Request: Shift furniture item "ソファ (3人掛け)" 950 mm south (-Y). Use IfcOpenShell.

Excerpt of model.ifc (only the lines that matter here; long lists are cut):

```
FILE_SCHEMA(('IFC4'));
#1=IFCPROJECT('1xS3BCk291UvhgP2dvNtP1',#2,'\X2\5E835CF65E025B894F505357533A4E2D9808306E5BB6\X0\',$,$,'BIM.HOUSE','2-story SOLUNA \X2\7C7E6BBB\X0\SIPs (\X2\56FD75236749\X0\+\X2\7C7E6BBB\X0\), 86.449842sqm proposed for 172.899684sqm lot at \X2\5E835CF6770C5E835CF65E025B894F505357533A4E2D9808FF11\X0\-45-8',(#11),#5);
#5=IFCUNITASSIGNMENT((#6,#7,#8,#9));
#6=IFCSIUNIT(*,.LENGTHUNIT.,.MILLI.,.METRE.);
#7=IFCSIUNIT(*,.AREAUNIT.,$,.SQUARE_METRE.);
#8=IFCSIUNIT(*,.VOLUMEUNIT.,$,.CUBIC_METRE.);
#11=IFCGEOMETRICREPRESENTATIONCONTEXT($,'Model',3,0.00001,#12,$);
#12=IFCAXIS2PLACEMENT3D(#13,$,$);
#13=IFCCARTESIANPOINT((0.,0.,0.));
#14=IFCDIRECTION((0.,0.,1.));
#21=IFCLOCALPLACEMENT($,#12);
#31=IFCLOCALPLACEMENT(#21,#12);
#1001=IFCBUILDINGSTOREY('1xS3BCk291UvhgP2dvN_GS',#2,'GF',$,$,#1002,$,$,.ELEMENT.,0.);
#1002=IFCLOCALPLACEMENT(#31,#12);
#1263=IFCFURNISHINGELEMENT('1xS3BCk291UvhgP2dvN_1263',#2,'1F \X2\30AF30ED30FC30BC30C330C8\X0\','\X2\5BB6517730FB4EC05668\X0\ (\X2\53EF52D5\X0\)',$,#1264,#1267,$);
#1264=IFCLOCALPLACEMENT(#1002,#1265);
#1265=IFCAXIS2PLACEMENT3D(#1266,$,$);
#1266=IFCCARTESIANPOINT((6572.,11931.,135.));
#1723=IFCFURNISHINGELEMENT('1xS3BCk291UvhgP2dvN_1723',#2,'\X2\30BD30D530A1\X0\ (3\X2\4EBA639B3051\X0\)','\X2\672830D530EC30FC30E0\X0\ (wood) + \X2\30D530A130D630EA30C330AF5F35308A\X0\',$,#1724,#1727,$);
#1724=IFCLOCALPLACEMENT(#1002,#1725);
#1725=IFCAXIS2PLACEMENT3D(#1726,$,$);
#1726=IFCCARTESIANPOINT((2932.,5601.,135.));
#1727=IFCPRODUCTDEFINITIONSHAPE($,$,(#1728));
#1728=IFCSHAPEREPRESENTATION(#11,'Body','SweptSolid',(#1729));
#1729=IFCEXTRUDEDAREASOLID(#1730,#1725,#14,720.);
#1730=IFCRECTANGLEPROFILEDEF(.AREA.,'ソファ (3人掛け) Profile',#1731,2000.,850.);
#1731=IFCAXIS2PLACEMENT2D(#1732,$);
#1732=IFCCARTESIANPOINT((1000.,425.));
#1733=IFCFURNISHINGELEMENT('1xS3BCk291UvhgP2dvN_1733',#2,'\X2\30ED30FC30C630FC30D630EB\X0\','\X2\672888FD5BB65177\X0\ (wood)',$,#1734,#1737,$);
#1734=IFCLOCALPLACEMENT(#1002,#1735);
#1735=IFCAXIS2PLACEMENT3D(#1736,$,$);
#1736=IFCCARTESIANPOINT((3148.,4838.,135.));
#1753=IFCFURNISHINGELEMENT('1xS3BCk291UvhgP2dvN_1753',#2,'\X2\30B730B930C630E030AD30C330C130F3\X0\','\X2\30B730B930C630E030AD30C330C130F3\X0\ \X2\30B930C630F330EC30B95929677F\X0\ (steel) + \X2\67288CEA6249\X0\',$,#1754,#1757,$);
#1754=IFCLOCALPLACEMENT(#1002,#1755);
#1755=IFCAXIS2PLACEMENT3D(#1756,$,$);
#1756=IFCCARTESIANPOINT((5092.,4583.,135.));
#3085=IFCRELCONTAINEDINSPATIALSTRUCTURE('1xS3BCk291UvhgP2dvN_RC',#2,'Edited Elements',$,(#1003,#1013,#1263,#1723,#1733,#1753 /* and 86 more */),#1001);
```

```python
import ifcopenshell
import ifcopenshell.api.geometry
import ifcopenshell.util.placement

model = ifcopenshell.open("model.ifc")

item = model.by_guid("1xS3BCk291UvhgP2dvN_1723")
matrix = ifcopenshell.util.placement.get_local_placement(item.ObjectPlacement)
matrix[1, 3] -= 950.0
ifcopenshell.api.geometry.edit_object_placement(model, product=item, matrix=matrix, is_si=False)

print(ifcopenshell.util.placement.get_local_placement(item.ObjectPlacement).round(3) + 0.0)

model.write("model-out.ifc")
```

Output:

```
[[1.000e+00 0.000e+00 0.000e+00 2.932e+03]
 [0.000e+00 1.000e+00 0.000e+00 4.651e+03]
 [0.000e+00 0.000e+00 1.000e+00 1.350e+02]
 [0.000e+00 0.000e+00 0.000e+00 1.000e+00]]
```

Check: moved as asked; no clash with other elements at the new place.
